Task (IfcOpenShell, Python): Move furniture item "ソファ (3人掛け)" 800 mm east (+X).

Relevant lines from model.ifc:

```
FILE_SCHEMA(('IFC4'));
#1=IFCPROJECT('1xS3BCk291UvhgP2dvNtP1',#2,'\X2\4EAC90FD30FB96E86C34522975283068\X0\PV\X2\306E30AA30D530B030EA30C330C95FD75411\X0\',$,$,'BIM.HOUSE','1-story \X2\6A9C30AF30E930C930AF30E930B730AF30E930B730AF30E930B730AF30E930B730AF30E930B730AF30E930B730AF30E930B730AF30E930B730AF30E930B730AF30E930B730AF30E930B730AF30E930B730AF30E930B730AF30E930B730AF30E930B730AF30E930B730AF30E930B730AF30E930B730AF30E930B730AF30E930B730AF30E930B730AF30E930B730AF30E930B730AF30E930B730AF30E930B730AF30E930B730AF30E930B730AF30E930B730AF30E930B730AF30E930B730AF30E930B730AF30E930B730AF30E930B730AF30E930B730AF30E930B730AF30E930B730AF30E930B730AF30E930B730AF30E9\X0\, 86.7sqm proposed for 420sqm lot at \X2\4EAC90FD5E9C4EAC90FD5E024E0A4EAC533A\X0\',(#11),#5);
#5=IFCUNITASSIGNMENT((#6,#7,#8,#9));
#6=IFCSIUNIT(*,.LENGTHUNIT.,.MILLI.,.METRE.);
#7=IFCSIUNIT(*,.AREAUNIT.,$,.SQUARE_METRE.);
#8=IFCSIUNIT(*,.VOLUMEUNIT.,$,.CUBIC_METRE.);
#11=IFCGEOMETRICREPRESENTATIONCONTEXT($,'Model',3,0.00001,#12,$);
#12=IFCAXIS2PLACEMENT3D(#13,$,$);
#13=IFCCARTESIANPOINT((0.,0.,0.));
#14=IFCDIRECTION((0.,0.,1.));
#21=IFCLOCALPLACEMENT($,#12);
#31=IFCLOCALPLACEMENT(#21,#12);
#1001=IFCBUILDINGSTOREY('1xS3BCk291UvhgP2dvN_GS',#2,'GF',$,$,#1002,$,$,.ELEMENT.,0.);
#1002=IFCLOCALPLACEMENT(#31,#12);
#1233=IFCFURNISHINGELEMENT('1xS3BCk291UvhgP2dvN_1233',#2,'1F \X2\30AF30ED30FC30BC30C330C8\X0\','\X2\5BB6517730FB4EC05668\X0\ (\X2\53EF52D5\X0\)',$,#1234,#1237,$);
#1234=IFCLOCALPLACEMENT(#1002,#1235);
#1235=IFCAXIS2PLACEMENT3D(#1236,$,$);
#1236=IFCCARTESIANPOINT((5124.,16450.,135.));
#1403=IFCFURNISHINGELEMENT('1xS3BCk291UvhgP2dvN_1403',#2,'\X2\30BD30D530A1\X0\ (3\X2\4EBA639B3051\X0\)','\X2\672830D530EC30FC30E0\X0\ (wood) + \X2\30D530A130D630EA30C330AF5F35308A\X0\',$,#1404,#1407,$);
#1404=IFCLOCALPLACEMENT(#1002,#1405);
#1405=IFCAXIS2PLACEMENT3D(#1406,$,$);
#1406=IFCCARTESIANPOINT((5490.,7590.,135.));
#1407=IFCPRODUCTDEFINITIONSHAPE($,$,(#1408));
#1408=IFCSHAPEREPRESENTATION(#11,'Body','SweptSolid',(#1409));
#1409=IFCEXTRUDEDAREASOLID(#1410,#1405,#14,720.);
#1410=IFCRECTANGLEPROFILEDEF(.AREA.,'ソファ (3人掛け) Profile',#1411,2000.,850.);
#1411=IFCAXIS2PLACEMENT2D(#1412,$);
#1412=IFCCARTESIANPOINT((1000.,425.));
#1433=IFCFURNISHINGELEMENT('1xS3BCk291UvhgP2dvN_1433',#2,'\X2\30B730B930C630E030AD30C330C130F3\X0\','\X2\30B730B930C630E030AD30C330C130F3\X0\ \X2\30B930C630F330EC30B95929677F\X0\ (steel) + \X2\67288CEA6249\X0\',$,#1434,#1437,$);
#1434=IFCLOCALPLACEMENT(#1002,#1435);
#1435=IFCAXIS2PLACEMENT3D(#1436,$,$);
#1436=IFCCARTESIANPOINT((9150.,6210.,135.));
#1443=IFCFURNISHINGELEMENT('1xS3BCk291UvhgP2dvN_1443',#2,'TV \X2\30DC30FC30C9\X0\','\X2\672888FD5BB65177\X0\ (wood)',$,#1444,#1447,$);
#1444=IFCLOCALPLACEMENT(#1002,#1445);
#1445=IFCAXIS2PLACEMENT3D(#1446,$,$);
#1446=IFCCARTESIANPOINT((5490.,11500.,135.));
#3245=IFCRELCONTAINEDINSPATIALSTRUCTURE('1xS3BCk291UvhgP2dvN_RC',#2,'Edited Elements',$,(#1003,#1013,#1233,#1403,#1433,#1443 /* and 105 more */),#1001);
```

```python
import ifcopenshell
import ifcopenshell.api.geometry
import ifcopenshell.util.placement

model = ifcopenshell.open("model.ifc")

item = model.by_guid("1xS3BCk291UvhgP2dvN_1403")
matrix = ifcopenshell.util.placement.get_local_placement(item.ObjectPlacement)
matrix[0, 3] += 800.0
ifcopenshell.api.geometry.edit_object_placement(model, product=item, matrix=matrix, is_si=False)

print(ifcopenshell.util.placement.get_local_placement(item.ObjectPlacement).round(3) + 0.0)

model.write("model_rev.ifc")
```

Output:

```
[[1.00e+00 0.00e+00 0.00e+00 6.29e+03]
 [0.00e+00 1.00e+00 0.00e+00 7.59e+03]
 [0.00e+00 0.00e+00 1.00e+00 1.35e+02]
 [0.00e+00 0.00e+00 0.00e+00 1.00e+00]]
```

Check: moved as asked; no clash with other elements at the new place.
